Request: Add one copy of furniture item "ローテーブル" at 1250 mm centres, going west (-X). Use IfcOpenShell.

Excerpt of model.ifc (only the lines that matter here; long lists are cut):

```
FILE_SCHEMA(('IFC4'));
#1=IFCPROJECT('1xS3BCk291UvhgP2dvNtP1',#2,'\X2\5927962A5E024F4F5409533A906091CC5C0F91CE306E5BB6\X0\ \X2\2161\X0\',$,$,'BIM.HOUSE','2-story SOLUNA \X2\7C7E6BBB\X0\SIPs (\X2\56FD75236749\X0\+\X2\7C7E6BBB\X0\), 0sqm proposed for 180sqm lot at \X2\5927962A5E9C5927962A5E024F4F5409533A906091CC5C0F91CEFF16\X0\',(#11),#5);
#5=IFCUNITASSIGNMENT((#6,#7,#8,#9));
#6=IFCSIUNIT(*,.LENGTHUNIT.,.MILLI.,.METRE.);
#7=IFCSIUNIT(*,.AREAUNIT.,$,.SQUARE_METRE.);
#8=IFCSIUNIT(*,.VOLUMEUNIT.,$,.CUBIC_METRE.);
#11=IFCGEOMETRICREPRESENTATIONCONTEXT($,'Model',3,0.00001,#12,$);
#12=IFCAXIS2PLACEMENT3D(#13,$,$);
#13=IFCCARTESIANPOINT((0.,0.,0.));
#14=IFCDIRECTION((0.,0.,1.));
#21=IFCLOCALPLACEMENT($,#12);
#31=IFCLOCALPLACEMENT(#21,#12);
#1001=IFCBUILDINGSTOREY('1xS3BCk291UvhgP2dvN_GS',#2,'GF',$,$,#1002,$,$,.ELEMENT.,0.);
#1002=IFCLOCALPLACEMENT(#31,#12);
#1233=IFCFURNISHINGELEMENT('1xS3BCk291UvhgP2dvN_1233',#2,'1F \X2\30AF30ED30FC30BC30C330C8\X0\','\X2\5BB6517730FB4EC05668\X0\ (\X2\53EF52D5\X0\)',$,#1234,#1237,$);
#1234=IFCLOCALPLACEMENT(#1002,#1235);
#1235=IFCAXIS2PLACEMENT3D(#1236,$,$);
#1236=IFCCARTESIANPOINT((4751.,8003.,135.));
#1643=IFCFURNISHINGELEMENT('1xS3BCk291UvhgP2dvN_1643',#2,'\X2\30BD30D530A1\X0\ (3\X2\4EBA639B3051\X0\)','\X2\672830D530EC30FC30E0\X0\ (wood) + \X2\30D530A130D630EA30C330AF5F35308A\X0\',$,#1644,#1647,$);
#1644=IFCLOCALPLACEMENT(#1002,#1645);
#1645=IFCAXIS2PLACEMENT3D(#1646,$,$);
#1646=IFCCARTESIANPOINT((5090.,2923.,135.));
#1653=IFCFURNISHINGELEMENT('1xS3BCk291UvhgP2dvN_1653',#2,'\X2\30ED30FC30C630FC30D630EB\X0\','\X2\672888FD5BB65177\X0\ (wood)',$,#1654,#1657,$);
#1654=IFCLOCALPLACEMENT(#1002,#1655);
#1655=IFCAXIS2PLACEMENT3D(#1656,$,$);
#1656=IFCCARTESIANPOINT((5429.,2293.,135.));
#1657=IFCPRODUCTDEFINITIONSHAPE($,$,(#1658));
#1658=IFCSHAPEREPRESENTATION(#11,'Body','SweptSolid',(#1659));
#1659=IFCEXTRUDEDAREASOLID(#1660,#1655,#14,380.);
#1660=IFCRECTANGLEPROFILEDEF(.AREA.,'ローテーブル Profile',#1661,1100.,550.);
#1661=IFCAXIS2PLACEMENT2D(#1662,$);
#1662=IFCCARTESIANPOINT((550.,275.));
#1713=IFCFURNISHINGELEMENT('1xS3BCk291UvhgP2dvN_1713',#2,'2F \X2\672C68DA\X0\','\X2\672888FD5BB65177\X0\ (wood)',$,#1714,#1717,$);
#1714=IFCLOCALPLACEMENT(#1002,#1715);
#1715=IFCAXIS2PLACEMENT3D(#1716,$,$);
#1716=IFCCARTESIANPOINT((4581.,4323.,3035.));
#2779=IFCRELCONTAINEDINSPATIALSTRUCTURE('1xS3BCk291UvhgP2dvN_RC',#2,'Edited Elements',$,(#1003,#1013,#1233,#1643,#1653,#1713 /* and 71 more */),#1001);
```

```python
import numpy as np
import ifcopenshell
import ifcopenshell.api.geometry
import ifcopenshell.api.root
import ifcopenshell.util.element
import ifcopenshell.util.placement
import ifcopenshell.util.unit

model = ifcopenshell.open("model.ifc")
unit_scale = ifcopenshell.util.unit.calculate_unit_scale(model)


def reuse_history(source, copy):
    """copy_class also copies each property set's owner history, people and application; keep the originals."""
    for rel in copy.IsDefinedBy:
        if rel.is_a("IfcRelDefinesByProperties") and (history := rel.RelatingPropertyDefinition.OwnerHistory):
            rel.RelatingPropertyDefinition.OwnerHistory = source.OwnerHistory
            ifcopenshell.util.element.remove_deep2(model, history)


source = model.by_guid("1xS3BCk291UvhgP2dvN_1653")
base = ifcopenshell.util.placement.get_local_placement(source.ObjectPlacement)
step = np.array([-1.0, 0.0, 0.0]) * 1.25 / unit_scale

for i in range(1, 2):
    copy = ifcopenshell.api.root.copy_class(model, product=source)
    copy.Representation = ifcopenshell.util.element.copy_deep(
        model, source.Representation, exclude=["IfcGeometricRepresentationContext", "IfcRepresentationMap"]
    )
    reuse_history(source, copy)
    matrix = base.copy()
    matrix[:3, 3] += i * step
    print("added at", matrix[:3, 3].round(3) + 0.0)
    ifcopenshell.api.geometry.edit_object_placement(model, product=copy, matrix=matrix, is_si=False)

model.write("model_updated.ifc")
```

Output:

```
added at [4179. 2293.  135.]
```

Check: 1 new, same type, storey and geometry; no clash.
